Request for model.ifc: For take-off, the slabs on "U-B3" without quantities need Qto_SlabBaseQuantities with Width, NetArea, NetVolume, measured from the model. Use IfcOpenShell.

First a look at what the model holds.

```python
import ifcopenshell
import ifcopenshell.util.element
import ifcopenshell.util.unit

model = ifcopenshell.open("model.ifc")
print(model.schema)
for unit_type in ("LENGTHUNIT", "AREAUNIT", "VOLUMEUNIT"):
    print(unit_type, ifcopenshell.util.unit.calculate_unit_scale(model, unit_type))
storey = next(s for s in model.by_type("IfcBuildingStorey") if s.Name == "U-B3")
slabs = [e for e in ifcopenshell.util.element.get_decomposition(storey) if e.is_a("IfcSlab")]
for e in sorted(slabs, key=lambda e: e.id()):
    print(e.id(), e.is_a(), e.Name, list(ifcopenshell.util.element.get_psets(e, qtos_only=True)), sep=" | ")
```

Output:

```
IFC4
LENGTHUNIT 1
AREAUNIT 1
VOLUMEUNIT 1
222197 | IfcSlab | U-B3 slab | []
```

```python
import ifcopenshell
import ifcopenshell.api.pset
import ifcopenshell.geom
import ifcopenshell.util.element
import ifcopenshell.util.shape
import ifcopenshell.util.unit

model = ifcopenshell.open("model.ifc")
unit_scale = ifcopenshell.util.unit.calculate_unit_scale(model)
area_scale = ifcopenshell.util.unit.calculate_unit_scale(model, "AREAUNIT")
volume_scale = ifcopenshell.util.unit.calculate_unit_scale(model, "VOLUMEUNIT")
settings = ifcopenshell.geom.settings()

storey = next(s for s in model.by_type("IfcBuildingStorey") if s.Name == "U-B3")
slabs = [e for e in ifcopenshell.util.element.get_decomposition(storey) if e.is_a("IfcSlab")]

for e in sorted(slabs, key=lambda e: e.id()):
    if ifcopenshell.util.element.get_psets(e, qtos_only=True, should_inherit=False):
        continue
    # Geometry comes back in metres, in the element's own axes.
    shape = ifcopenshell.geom.create_shape(settings, e)
    values = {
        "Width": ifcopenshell.util.shape.get_z(shape.geometry) / unit_scale,
        "NetArea": ifcopenshell.util.shape.get_footprint_area(shape.geometry) / area_scale,
        "NetVolume": ifcopenshell.util.shape.get_volume(shape.geometry) / volume_scale,
    }
    qto = ifcopenshell.api.pset.add_qto(model, product=e, name="Qto_SlabBaseQuantities")
    ifcopenshell.api.pset.edit_qto(model, qto=qto, properties=values)
    print(e.id(), {k: round(v, 3) for k, v in values.items()})

model.write("model_v2.ifc")
```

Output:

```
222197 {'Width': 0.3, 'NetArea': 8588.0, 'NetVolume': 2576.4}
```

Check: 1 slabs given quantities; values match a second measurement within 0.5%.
